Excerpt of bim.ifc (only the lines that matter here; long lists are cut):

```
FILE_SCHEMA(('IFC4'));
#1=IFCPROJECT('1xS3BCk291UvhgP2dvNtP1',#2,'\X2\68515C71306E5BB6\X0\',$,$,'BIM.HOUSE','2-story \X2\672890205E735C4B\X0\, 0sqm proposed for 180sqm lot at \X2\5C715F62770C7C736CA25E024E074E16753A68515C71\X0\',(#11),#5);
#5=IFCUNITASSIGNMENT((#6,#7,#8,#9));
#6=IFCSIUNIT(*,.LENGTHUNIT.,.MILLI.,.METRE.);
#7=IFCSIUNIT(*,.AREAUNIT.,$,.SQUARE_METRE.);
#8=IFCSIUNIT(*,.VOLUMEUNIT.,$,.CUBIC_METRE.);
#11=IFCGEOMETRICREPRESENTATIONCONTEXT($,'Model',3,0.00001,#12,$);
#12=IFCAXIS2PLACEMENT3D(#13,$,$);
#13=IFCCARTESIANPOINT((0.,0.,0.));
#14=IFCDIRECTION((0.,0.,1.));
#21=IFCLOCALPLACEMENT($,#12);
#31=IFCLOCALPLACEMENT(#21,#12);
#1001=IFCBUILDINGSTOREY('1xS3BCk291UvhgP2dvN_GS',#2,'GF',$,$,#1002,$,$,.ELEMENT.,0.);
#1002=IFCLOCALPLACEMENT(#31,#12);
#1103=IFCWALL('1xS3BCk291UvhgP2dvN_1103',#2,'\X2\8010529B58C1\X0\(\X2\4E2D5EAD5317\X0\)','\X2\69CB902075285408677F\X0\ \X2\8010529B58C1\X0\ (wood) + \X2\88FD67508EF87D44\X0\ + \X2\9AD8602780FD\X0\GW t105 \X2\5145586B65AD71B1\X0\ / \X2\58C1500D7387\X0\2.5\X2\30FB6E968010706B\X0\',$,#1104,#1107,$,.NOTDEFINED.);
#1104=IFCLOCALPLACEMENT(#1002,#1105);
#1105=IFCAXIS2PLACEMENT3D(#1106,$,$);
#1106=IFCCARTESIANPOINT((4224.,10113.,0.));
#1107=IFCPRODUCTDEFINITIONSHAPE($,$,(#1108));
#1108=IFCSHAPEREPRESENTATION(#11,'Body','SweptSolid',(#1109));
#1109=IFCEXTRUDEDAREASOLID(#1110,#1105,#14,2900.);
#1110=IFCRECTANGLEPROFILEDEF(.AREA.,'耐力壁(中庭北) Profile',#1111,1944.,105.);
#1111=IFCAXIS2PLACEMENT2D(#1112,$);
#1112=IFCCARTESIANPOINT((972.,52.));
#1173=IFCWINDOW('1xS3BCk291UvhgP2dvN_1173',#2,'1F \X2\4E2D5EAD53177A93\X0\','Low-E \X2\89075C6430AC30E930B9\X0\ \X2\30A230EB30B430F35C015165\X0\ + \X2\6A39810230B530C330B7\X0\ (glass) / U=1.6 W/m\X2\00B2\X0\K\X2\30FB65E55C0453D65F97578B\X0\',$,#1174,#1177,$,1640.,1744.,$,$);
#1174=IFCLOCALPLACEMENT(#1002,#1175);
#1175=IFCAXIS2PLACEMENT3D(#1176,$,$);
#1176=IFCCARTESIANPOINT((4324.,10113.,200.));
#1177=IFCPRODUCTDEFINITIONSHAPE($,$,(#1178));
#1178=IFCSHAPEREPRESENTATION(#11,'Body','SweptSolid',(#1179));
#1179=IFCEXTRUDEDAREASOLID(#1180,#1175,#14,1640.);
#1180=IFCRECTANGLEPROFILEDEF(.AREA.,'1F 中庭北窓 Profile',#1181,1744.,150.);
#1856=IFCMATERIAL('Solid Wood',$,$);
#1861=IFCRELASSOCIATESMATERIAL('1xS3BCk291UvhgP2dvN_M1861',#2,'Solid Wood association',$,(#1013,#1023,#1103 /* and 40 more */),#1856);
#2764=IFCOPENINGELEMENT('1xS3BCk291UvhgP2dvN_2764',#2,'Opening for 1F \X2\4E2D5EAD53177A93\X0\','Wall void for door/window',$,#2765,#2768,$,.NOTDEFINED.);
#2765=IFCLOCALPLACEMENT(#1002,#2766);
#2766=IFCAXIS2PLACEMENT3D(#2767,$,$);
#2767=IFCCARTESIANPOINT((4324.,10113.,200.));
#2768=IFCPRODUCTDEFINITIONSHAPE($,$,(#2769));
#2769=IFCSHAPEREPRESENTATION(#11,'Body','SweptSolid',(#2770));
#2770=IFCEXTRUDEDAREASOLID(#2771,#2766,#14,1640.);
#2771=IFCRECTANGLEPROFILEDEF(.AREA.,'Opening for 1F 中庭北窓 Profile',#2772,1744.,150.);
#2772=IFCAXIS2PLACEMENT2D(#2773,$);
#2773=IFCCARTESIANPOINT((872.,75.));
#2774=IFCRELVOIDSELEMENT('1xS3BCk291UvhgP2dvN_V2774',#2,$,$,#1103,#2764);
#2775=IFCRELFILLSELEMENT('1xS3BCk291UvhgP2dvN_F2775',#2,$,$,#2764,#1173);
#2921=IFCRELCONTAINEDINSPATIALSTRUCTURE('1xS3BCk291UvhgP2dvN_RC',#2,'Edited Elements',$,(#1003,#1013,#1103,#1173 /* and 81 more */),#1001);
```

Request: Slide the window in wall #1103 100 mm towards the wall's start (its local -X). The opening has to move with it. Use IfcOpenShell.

```python
import ifcopenshell
import ifcopenshell.api.geometry
import ifcopenshell.util.placement

model = ifcopenshell.open("bim.ifc")

window = model.by_guid("1xS3BCk291UvhgP2dvN_1173")
opening = window.FillsVoids[0].RelatingOpeningElement
wall = opening.VoidsElements[0].RelatingBuildingElement

wall_matrix = ifcopenshell.util.placement.get_local_placement(wall.ObjectPlacement)
shift = wall_matrix[:3, 0] * -100.0
before = ifcopenshell.util.placement.get_local_placement(window.ObjectPlacement)[:3, 3].copy()

# The window is not placed relative to its opening, so move both.
for product in (opening, window):
    matrix = ifcopenshell.util.placement.get_local_placement(product.ObjectPlacement)
    matrix[:3, 3] += shift
    ifcopenshell.api.geometry.edit_object_placement(model, product=product, matrix=matrix, is_si=False)

after = ifcopenshell.util.placement.get_local_placement(window.ObjectPlacement)[:3, 3]
print("window moved by", (after - before).round(3) + 0.0)

model.write("bim_v2.ifc")
```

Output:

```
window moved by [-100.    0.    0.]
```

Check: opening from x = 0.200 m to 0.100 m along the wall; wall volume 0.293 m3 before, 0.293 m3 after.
